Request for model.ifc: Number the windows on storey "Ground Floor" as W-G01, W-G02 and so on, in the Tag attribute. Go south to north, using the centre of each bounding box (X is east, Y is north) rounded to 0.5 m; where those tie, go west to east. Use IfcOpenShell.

First a look at what the model holds.

```python
import ifcopenshell
import ifcopenshell.util.element
import ifcopenshell.util.placement

model = ifcopenshell.open("model.ifc")
print(model.schema)
storey = next(s for s in model.by_type("IfcBuildingStorey") if s.Name == "Ground Floor")
windows = [e for e in ifcopenshell.util.element.get_decomposition(storey) if e.is_a("IfcWindow")]
for e in sorted(windows, key=lambda e: e.id()):
    origin = ifcopenshell.util.placement.get_local_placement(e.ObjectPlacement)[:3, 3]
    print(e.id(), e.Tag, e.Name, origin.round(2) + 0.0, sep=" | ")
```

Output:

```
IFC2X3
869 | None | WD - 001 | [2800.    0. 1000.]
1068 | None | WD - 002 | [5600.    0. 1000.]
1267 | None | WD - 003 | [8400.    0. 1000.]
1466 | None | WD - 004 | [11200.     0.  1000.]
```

```python
import ifcopenshell
import ifcopenshell.geom
import ifcopenshell.util.element
import ifcopenshell.util.shape

model = ifcopenshell.open("model.ifc")
settings = ifcopenshell.geom.settings()
settings.set("use-world-coords", True)


def centre(element):
    shape = ifcopenshell.geom.create_shape(settings, element)
    return ifcopenshell.util.shape.get_bbox_centroid(shape.geometry)


storey = next(s for s in model.by_type("IfcBuildingStorey") if s.Name == "Ground Floor")
windows = [e for e in ifcopenshell.util.element.get_decomposition(storey) if e.is_a("IfcWindow")]

# Insertion points can sit at a corner or the storey origin, so sort by the geometry (in metres).
centres = {e: centre(e) for e in windows}
windows.sort(key=lambda e: (round(centres[e][1] / 0.5), centres[e][0]))

for i, e in enumerate(windows, start=1):
    number = f"W-G{i:02d}"
    e.Tag = number
    print(e.id(), number)

model.write("model_rev.ifc")
```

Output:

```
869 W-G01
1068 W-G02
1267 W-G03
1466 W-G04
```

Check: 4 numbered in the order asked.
